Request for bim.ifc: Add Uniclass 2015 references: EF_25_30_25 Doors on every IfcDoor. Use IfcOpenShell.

First a look at what the model holds.

```python
import ifcopenshell

model = ifcopenshell.open("bim.ifc")
print(model.schema)
print("classifications:", [c.Name for c in model.by_type("IfcClassification")])
for ifc_class in ("IfcDoor", "IfcRoof", "IfcStair", "IfcWall", "IfcWindow"):
    print(ifc_class, len(model.by_type(ifc_class)))
```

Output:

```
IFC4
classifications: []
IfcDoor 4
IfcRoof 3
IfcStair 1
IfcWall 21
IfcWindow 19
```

```python
import ifcopenshell
import ifcopenshell.api.classification

model = ifcopenshell.open("bim.ifc")

system = ifcopenshell.api.classification.add_classification(model, classification="Uniclass 2015")

codes = {
    "IfcDoor": ("EF_25_30_25", "Doors"),
}
for ifc_class, (code, name) in codes.items():
    products = model.by_type(ifc_class)
    ifcopenshell.api.classification.add_reference(
        model, products=products, classification=system, identification=code, name=name
    )
    print(code, len(products))

model.write("bim_edited.ifc")
```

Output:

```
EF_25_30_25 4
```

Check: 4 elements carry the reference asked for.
